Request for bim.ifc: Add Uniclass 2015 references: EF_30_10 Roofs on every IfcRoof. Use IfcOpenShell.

First a look at what the model holds.

```python
import ifcopenshell

model = ifcopenshell.open("bim.ifc")
print(model.schema)
print("classifications:", [c.Name for c in model.by_type("IfcClassification")])
for ifc_class in ("IfcDoor", "IfcRoof", "IfcStair", "IfcWall", "IfcWindow"):
    print(ifc_class, len(model.by_type(ifc_class)))
```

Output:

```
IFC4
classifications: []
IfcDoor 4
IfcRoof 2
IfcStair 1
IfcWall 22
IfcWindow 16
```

```python
import ifcopenshell
import ifcopenshell.api.classification

model = ifcopenshell.open("bim.ifc")

system = ifcopenshell.api.classification.add_classification(model, classification="Uniclass 2015")

codes = {
    "IfcRoof": ("EF_30_10", "Roofs"),
}
for ifc_class, (code, name) in codes.items():
    products = model.by_type(ifc_class)
    ifcopenshell.api.classification.add_reference(
        model, products=products, classification=system, identification=code, name=name
    )
    print(code, len(products))

model.write("bim_v2.ifc")
```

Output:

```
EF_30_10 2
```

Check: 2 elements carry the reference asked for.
